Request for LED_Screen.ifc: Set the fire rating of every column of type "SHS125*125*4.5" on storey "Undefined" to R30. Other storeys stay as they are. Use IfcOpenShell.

First a look at what the model holds.

```python
import ifcopenshell
import ifcopenshell.util.element

model = ifcopenshell.open("LED_Screen.ifc")
print(model.schema)
storey = next(s for s in model.by_type("IfcBuildingStorey") if s.Name == "Undefined")
columns = [e for e in ifcopenshell.util.element.get_decomposition(storey) if e.is_a("IfcColumn")]
seen = {}
for e in columns:
    element_type = ifcopenshell.util.element.get_type(e)
    key = (element_type.Name if element_type != e and element_type else None, ifcopenshell.util.element.get_pset(e, "Pset_ColumnCommon", "FireRating"))
    seen[key] = seen.get(key, 0) + 1
for (name, value), count in sorted(seen.items(), key=str):
    print(count, "x", name, "|", value)
```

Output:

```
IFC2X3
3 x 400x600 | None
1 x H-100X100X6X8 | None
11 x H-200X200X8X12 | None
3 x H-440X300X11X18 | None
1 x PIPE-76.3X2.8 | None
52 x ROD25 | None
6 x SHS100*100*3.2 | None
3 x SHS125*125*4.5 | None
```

```python
import ifcopenshell
import ifcopenshell.api.pset
import ifcopenshell.util.element

model = ifcopenshell.open("LED_Screen.ifc")

storey = next(s for s in model.by_type("IfcBuildingStorey") if s.Name == "Undefined")
columns = [e for e in ifcopenshell.util.element.get_decomposition(storey) if e.is_a("IfcColumn")]

count = 0
for e in columns:
    element_type = ifcopenshell.util.element.get_type(e)
    if element_type in (None, e) or element_type.Name != "SHS125*125*4.5":
        continue
    found = ifcopenshell.util.element.get_pset(e, "Pset_ColumnCommon", should_inherit=False)
    if found:
        pset = model.by_id(found["id"])
        if len(ifcopenshell.util.element.get_elements_by_pset(pset)) > 1:
            pset = ifcopenshell.api.pset.unshare_pset(model, products=[e], pset=pset)[0]
    else:
        pset = ifcopenshell.api.pset.add_pset(model, product=e, name="Pset_ColumnCommon")
    ifcopenshell.api.pset.edit_pset(model, pset=pset, properties={"FireRating": "R30"})
    count += 1

print(count, "columns updated")

model.write("LED_Screen_v2.ifc")
```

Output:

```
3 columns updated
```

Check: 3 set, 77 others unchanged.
